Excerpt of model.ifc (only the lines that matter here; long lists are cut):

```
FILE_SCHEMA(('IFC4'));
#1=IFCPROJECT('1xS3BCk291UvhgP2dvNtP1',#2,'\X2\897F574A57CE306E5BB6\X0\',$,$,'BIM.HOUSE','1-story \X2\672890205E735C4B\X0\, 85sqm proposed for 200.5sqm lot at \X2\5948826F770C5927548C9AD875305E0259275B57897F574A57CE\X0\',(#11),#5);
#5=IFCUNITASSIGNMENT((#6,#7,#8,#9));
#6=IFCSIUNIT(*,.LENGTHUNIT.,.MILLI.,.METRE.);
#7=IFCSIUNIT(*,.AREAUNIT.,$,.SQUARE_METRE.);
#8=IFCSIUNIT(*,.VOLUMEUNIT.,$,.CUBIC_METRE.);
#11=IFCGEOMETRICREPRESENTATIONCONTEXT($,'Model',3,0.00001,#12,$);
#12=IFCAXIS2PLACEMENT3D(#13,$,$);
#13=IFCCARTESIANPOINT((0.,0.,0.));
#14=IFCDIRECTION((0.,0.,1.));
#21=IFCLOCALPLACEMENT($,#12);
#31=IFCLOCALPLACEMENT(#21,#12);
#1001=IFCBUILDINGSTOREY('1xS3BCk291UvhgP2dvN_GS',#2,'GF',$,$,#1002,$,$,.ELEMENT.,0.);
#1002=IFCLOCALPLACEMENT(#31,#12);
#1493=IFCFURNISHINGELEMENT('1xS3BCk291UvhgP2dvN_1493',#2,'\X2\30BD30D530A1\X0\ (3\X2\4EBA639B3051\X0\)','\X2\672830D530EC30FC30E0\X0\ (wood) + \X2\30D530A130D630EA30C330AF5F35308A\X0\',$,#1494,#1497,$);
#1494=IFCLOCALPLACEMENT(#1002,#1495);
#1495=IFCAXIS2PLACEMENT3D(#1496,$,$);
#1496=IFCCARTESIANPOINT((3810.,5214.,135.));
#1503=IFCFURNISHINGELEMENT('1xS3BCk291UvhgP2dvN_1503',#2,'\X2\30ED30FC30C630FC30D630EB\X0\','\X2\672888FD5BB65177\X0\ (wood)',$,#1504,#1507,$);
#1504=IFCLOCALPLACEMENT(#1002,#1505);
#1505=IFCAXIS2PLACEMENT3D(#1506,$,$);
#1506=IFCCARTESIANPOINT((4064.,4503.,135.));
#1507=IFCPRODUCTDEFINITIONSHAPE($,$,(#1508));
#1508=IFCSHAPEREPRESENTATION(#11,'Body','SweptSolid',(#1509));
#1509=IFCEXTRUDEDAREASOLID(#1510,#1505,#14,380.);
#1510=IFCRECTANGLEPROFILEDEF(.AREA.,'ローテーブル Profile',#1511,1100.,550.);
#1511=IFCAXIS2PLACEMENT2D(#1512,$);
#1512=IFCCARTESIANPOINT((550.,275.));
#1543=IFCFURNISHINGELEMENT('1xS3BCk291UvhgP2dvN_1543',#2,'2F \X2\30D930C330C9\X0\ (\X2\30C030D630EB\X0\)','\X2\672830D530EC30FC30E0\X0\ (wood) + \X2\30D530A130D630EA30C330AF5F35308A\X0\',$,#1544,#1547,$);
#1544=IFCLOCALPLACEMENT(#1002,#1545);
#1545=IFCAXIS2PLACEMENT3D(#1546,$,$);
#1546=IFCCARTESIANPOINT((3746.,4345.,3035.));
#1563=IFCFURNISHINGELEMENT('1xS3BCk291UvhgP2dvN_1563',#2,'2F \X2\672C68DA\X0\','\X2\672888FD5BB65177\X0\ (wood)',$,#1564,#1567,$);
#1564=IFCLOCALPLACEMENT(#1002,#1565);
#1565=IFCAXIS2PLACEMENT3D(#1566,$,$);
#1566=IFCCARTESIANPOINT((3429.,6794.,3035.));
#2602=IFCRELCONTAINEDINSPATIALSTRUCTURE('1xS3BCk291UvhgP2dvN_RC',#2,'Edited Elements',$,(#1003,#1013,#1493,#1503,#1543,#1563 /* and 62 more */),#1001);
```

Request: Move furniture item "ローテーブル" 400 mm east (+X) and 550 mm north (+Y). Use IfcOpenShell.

```python
import ifcopenshell
import ifcopenshell.api.geometry
import ifcopenshell.util.placement

model = ifcopenshell.open("model.ifc")

item = model.by_guid("1xS3BCk291UvhgP2dvN_1503")
matrix = ifcopenshell.util.placement.get_local_placement(item.ObjectPlacement)
matrix[0, 3] += 400.0
matrix[1, 3] += 550.0
ifcopenshell.api.geometry.edit_object_placement(model, product=item, matrix=matrix, is_si=False)

print(ifcopenshell.util.placement.get_local_placement(item.ObjectPlacement).round(3) + 0.0)

model.write("model_edited.ifc")
```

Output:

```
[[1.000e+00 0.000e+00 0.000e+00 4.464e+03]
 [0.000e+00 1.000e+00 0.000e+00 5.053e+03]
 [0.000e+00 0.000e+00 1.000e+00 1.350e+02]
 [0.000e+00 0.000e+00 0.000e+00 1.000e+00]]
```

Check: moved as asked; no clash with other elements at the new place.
